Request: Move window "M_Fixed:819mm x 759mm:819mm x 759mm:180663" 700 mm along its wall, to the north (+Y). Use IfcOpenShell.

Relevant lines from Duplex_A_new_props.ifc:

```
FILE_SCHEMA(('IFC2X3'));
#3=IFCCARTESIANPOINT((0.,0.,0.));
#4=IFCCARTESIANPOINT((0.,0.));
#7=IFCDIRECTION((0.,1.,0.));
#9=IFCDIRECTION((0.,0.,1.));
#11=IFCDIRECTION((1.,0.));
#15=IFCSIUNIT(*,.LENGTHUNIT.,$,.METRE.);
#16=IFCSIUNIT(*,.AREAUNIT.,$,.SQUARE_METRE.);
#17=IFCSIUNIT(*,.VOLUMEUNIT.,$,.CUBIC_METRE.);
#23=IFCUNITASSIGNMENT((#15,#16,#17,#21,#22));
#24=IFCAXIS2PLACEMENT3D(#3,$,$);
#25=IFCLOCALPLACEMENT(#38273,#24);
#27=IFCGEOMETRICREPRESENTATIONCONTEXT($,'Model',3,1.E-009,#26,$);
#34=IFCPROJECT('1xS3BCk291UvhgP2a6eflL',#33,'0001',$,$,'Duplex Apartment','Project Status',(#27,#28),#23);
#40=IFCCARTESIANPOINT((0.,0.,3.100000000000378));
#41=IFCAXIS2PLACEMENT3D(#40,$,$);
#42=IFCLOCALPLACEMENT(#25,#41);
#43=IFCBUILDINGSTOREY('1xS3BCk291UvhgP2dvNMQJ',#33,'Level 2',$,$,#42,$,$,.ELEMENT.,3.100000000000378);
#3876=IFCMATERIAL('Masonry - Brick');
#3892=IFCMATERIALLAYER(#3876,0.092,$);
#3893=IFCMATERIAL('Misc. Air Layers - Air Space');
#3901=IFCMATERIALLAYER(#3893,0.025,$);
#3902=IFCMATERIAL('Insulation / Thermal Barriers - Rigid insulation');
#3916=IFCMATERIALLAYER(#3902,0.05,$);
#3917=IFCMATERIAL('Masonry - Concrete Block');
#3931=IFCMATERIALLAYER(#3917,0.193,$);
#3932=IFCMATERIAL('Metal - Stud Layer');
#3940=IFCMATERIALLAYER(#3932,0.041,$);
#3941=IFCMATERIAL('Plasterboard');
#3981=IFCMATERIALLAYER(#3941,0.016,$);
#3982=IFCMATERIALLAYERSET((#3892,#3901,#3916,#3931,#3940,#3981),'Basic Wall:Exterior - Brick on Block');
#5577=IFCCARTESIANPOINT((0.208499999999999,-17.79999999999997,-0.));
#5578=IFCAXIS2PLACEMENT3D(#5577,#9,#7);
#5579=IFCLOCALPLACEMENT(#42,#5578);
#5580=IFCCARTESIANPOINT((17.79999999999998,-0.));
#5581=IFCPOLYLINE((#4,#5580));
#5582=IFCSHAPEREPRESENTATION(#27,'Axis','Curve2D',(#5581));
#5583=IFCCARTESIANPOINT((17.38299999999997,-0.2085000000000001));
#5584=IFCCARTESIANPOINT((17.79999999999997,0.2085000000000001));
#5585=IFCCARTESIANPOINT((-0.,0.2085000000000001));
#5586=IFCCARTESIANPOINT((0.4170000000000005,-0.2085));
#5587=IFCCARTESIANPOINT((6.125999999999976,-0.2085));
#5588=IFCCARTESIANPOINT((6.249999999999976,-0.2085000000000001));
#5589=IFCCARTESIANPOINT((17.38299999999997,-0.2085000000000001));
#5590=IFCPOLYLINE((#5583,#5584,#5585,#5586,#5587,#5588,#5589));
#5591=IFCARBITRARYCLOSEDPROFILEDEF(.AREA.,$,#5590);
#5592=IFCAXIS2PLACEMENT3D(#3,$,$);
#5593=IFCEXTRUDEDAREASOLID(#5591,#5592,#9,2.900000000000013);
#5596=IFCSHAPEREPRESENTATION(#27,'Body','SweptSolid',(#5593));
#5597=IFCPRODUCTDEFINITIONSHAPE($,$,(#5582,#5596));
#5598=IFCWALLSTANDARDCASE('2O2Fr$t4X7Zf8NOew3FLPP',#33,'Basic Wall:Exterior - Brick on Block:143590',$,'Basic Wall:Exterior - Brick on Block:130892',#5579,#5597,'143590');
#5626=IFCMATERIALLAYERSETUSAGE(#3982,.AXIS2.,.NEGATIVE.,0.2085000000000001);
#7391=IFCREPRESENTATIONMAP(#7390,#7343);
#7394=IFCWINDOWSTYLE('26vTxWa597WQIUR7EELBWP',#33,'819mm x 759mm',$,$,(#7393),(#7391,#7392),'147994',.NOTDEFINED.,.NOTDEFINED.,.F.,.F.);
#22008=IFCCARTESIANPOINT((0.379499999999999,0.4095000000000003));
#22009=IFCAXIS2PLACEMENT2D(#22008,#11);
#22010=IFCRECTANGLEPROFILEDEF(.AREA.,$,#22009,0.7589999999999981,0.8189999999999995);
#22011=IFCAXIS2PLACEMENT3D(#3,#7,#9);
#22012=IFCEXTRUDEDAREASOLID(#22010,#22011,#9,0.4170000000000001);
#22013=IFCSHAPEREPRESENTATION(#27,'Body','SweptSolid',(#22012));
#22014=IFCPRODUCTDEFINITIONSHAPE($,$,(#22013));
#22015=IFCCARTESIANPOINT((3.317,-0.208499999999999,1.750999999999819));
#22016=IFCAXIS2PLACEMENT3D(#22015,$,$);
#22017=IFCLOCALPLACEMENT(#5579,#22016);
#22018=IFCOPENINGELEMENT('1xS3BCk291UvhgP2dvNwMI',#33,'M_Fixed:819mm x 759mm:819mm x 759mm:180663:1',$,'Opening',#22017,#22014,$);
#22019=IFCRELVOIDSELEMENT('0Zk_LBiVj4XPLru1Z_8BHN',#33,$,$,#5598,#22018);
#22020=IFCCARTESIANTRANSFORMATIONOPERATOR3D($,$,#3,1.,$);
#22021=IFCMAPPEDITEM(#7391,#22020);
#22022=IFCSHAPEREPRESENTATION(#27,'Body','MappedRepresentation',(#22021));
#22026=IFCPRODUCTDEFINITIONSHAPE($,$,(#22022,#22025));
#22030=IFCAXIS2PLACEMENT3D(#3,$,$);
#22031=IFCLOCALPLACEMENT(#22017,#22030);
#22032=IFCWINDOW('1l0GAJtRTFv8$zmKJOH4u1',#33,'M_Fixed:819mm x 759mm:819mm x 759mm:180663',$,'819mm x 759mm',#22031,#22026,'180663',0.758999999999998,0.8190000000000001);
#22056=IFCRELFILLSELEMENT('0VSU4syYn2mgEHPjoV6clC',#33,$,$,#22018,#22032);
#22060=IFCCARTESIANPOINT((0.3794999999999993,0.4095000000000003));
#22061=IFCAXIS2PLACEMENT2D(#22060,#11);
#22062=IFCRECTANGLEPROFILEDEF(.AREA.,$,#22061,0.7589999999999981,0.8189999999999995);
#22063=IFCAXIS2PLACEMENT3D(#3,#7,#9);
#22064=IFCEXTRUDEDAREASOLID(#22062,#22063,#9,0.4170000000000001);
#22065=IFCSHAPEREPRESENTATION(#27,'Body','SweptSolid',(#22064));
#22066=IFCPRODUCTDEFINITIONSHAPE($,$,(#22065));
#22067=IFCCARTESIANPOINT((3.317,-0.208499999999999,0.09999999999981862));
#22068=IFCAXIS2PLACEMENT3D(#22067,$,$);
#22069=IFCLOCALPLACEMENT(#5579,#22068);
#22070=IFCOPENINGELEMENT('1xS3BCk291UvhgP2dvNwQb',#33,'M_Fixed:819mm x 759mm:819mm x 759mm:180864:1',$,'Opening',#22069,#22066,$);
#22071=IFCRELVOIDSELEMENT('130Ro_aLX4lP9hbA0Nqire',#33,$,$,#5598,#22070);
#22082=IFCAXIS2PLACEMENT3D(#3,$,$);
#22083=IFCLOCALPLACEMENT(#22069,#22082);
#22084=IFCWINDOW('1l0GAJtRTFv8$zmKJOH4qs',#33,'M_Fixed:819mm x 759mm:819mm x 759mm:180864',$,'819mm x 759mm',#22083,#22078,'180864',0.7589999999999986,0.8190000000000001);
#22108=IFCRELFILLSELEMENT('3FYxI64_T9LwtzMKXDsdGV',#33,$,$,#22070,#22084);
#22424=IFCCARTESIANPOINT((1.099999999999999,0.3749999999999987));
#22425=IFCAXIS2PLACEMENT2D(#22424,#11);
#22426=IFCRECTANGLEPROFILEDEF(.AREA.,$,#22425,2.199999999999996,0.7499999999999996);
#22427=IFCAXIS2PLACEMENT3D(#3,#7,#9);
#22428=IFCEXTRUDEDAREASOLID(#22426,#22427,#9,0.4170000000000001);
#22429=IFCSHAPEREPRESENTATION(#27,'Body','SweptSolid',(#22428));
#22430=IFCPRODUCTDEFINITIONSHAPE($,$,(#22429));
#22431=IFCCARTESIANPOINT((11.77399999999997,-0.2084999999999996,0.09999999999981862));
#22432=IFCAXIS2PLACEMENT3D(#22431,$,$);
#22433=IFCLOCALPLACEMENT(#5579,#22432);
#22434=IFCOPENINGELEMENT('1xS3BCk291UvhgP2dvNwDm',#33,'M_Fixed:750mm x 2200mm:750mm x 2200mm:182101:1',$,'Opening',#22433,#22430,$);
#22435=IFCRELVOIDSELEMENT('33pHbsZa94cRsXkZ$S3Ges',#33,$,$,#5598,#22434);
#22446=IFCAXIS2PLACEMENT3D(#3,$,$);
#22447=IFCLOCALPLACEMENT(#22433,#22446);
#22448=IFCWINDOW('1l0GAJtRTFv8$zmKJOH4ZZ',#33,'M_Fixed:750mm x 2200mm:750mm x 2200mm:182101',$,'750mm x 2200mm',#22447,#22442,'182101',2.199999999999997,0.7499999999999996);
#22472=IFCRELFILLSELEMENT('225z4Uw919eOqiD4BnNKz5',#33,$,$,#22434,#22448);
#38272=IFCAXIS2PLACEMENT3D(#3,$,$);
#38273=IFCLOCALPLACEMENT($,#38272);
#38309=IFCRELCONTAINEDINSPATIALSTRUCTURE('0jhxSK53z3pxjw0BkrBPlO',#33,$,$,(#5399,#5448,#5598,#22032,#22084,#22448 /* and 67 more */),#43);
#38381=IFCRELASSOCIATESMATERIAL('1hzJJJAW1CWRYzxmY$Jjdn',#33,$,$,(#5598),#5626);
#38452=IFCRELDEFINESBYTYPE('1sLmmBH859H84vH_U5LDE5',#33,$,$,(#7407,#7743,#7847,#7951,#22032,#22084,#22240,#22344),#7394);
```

```python
import ifcopenshell
import ifcopenshell.api.geometry
import ifcopenshell.util.placement

model = ifcopenshell.open("Duplex_A_new_props.ifc")

window = model.by_id(22032)
opening = window.FillsVoids[0].RelatingOpeningElement
wall = opening.VoidsElements[0].RelatingBuildingElement

wall_matrix = ifcopenshell.util.placement.get_local_placement(wall.ObjectPlacement)
shift = wall_matrix[:3, 0] * 0.7
before = ifcopenshell.util.placement.get_local_placement(window.ObjectPlacement)[:3, 3].copy()

# The window is placed relative to its opening, so it follows when the opening moves.
matrix = ifcopenshell.util.placement.get_local_placement(opening.ObjectPlacement)
matrix[:3, 3] += shift
ifcopenshell.api.geometry.edit_object_placement(
    model, product=opening, matrix=matrix, is_si=False, should_transform_children=True
)

after = ifcopenshell.util.placement.get_local_placement(window.ObjectPlacement)[:3, 3]
print("window moved by", (after - before).round(3) + 0.0)

model.write("Duplex_A_new_props_updated.ifc")
```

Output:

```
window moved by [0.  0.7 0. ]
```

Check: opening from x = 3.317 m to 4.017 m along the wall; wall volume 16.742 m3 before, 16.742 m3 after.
